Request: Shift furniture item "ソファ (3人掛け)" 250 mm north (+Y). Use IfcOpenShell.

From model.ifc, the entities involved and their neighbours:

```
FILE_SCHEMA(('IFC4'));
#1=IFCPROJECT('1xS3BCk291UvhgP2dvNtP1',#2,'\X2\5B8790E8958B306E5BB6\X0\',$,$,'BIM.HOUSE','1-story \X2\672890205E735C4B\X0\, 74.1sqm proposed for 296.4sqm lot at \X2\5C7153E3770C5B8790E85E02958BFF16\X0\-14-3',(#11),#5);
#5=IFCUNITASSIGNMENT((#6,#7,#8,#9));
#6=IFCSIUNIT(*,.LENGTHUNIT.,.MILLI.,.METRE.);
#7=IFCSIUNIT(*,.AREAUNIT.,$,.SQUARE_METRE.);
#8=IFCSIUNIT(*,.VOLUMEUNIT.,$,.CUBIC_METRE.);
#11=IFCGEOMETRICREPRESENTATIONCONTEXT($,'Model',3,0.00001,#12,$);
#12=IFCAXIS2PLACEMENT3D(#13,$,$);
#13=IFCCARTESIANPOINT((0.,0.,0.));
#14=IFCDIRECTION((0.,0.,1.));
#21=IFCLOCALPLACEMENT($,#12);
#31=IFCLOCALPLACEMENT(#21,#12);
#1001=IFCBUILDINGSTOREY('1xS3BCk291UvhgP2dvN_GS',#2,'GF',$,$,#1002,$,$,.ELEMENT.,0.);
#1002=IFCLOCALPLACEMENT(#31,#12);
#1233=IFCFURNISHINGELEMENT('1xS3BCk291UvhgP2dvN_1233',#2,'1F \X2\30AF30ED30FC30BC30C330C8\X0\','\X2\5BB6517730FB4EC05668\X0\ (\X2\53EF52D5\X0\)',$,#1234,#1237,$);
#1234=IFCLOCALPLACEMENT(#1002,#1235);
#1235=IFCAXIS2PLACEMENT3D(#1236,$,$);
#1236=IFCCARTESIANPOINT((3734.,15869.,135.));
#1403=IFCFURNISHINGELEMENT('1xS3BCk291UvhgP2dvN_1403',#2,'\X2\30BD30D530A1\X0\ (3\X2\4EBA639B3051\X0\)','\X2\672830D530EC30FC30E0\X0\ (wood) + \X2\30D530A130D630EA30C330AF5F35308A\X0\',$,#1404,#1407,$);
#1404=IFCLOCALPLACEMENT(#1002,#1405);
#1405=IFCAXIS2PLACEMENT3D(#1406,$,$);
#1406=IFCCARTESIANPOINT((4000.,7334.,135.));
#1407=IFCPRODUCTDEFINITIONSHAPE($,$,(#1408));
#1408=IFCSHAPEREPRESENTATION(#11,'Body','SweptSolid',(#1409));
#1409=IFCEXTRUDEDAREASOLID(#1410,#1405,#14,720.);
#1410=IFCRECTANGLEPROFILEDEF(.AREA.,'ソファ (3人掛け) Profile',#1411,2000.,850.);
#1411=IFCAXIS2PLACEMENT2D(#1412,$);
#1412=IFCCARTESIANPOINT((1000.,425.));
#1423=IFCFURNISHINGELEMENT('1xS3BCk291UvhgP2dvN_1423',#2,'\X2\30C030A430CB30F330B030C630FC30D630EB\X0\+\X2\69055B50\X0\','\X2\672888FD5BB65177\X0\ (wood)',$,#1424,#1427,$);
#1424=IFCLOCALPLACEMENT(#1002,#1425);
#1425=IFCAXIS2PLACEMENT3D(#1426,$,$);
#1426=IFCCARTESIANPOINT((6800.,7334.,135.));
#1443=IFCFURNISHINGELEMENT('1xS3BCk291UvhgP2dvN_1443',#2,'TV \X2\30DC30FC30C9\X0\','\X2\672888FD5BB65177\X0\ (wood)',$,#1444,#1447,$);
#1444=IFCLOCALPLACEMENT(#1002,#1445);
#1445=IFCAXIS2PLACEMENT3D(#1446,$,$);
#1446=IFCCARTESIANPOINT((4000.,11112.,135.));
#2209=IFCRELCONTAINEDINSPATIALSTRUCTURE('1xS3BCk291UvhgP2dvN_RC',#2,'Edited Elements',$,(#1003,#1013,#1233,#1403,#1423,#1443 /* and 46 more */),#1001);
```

```python
import ifcopenshell
import ifcopenshell.api.geometry
import ifcopenshell.util.placement

model = ifcopenshell.open("model.ifc")

item = model.by_guid("1xS3BCk291UvhgP2dvN_1403")
matrix = ifcopenshell.util.placement.get_local_placement(item.ObjectPlacement)
matrix[1, 3] += 250.0
ifcopenshell.api.geometry.edit_object_placement(model, product=item, matrix=matrix, is_si=False)

print(ifcopenshell.util.placement.get_local_placement(item.ObjectPlacement).round(3) + 0.0)

model.write("model_edited.ifc")
```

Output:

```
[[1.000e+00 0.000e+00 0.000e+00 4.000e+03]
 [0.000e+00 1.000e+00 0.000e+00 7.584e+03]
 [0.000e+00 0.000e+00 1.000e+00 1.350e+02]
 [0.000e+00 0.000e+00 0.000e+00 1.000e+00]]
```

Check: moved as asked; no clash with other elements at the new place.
